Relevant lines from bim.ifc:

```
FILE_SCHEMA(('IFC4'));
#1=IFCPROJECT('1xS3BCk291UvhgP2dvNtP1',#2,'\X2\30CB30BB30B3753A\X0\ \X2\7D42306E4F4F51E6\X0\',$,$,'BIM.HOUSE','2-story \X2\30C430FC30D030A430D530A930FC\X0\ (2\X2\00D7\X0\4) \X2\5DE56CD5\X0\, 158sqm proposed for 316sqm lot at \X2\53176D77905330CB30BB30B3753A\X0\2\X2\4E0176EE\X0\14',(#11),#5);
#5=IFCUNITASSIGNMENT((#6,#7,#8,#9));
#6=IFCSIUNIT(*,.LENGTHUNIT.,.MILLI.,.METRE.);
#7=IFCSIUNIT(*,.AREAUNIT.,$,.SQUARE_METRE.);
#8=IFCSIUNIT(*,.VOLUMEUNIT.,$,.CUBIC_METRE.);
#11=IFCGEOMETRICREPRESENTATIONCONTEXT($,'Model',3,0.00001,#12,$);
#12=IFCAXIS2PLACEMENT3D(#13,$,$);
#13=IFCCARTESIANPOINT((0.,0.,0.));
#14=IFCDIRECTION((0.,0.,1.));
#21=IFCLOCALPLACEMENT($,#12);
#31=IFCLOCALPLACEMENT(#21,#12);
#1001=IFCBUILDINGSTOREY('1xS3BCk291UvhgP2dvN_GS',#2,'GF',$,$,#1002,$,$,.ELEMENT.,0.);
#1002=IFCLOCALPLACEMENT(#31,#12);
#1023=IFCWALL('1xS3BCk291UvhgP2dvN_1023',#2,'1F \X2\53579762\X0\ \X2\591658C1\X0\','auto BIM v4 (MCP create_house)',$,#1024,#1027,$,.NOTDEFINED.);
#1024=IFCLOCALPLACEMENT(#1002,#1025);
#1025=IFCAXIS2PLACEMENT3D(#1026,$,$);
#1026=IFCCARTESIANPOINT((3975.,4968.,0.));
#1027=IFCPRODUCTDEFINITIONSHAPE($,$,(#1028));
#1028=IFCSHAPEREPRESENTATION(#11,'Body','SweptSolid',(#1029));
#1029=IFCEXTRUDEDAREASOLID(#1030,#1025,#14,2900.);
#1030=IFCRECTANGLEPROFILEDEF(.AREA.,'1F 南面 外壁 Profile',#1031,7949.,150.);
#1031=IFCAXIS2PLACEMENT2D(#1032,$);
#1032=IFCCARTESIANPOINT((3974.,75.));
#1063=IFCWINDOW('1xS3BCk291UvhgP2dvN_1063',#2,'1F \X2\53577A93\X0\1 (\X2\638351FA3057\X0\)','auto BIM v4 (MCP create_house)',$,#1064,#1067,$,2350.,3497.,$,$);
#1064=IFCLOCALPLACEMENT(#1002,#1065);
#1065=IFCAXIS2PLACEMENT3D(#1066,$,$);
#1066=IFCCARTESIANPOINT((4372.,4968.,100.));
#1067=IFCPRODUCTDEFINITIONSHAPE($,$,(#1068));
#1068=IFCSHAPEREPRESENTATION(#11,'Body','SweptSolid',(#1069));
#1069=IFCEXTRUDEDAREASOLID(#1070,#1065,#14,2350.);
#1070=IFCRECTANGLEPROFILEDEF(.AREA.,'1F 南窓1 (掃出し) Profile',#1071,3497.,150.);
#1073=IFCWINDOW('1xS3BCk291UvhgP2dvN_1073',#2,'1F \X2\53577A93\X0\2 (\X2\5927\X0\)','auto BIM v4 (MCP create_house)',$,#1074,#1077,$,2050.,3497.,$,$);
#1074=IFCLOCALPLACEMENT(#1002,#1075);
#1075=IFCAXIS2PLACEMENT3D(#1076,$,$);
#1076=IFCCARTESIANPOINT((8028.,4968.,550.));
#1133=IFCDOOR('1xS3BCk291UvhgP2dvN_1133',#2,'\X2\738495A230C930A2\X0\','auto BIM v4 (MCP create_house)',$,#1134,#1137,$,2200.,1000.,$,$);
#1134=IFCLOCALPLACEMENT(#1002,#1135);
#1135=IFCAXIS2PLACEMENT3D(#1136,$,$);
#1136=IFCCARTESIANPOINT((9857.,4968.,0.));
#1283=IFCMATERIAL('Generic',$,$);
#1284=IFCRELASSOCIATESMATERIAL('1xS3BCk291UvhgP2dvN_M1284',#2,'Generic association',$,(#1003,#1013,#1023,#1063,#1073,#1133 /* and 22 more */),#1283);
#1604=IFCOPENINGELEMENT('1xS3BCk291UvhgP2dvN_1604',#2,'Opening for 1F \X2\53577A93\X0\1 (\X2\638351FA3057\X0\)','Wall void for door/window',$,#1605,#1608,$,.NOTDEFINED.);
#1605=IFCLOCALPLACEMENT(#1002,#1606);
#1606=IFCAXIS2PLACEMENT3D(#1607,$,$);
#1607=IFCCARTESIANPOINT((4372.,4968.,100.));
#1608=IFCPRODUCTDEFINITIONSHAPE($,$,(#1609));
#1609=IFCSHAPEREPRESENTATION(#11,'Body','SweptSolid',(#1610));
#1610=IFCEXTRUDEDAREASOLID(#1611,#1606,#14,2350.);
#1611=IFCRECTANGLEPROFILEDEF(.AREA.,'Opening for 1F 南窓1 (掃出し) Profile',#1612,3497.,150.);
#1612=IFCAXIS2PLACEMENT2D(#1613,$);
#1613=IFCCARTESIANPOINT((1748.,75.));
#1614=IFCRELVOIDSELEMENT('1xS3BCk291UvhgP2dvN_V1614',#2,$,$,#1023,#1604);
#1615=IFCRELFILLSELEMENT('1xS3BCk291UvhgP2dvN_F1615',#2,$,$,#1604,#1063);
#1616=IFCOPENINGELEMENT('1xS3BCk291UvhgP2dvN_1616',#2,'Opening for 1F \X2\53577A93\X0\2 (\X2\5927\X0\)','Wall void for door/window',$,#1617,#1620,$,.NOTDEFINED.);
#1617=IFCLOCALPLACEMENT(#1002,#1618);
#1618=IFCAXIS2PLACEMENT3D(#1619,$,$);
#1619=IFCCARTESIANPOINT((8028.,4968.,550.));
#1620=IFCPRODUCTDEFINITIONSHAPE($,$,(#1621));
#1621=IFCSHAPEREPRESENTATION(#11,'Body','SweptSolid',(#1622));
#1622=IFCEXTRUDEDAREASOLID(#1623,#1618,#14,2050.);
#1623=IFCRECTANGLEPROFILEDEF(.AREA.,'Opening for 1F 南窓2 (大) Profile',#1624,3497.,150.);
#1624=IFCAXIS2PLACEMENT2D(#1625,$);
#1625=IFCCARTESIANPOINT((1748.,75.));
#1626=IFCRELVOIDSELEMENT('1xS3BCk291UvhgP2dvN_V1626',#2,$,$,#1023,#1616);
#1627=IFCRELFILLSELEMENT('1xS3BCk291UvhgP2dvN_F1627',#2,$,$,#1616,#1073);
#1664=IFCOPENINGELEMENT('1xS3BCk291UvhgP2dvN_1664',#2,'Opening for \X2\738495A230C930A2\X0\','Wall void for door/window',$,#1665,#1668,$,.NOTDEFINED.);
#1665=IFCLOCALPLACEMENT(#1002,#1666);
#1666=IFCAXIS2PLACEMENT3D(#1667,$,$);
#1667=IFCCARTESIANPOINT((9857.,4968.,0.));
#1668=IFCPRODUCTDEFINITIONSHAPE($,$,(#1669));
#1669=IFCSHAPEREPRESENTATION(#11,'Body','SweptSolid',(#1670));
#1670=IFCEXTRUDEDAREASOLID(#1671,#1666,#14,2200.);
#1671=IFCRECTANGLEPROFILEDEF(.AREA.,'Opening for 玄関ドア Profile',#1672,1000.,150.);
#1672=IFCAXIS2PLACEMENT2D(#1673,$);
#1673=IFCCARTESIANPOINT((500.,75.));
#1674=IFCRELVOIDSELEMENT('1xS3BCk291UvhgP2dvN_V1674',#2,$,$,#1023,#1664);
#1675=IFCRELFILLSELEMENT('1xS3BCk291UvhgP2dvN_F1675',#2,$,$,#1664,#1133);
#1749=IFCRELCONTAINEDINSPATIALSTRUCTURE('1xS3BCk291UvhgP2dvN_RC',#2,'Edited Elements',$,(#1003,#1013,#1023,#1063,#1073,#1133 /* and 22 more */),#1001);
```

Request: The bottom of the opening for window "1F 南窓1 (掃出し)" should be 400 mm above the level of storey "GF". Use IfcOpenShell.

```python
import numpy as np
import ifcopenshell
import ifcopenshell.api.geometry
import ifcopenshell.geom
import ifcopenshell.util.element
import ifcopenshell.util.placement
import ifcopenshell.util.shape
import ifcopenshell.util.unit

model = ifcopenshell.open("bim.ifc")
unit_scale = ifcopenshell.util.unit.calculate_unit_scale(model)

window = model.by_guid("1xS3BCk291UvhgP2dvN_1063")
opening = window.FillsVoids[0].RelatingOpeningElement
storey = ifcopenshell.util.element.get_container(window, ifc_class="IfcBuildingStorey")
level = ifcopenshell.util.placement.get_local_placement(storey.ObjectPlacement)[2, 3]

# The opening's origin need not be at the sill, so measure its lowest point.
shape = ifcopenshell.geom.create_shape(ifcopenshell.geom.settings(), opening)
bottom = ifcopenshell.util.shape.get_shape_bottom_elevation(shape, shape.geometry) / unit_scale
dz = level + 0.4 / unit_scale - bottom

shift = np.array([0.0, 0.0, dz])
# The window is not placed relative to its opening, so move both.
for product in (opening, window):
    matrix = ifcopenshell.util.placement.get_local_placement(product.ObjectPlacement)
    matrix[:3, 3] += shift
    ifcopenshell.api.geometry.edit_object_placement(model, product=product, matrix=matrix, is_si=False)

print(f"moved by {dz * unit_scale:+.3f} m")

model.write("bim_v2.ifc")
```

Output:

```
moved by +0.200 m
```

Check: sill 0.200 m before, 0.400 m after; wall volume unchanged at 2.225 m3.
